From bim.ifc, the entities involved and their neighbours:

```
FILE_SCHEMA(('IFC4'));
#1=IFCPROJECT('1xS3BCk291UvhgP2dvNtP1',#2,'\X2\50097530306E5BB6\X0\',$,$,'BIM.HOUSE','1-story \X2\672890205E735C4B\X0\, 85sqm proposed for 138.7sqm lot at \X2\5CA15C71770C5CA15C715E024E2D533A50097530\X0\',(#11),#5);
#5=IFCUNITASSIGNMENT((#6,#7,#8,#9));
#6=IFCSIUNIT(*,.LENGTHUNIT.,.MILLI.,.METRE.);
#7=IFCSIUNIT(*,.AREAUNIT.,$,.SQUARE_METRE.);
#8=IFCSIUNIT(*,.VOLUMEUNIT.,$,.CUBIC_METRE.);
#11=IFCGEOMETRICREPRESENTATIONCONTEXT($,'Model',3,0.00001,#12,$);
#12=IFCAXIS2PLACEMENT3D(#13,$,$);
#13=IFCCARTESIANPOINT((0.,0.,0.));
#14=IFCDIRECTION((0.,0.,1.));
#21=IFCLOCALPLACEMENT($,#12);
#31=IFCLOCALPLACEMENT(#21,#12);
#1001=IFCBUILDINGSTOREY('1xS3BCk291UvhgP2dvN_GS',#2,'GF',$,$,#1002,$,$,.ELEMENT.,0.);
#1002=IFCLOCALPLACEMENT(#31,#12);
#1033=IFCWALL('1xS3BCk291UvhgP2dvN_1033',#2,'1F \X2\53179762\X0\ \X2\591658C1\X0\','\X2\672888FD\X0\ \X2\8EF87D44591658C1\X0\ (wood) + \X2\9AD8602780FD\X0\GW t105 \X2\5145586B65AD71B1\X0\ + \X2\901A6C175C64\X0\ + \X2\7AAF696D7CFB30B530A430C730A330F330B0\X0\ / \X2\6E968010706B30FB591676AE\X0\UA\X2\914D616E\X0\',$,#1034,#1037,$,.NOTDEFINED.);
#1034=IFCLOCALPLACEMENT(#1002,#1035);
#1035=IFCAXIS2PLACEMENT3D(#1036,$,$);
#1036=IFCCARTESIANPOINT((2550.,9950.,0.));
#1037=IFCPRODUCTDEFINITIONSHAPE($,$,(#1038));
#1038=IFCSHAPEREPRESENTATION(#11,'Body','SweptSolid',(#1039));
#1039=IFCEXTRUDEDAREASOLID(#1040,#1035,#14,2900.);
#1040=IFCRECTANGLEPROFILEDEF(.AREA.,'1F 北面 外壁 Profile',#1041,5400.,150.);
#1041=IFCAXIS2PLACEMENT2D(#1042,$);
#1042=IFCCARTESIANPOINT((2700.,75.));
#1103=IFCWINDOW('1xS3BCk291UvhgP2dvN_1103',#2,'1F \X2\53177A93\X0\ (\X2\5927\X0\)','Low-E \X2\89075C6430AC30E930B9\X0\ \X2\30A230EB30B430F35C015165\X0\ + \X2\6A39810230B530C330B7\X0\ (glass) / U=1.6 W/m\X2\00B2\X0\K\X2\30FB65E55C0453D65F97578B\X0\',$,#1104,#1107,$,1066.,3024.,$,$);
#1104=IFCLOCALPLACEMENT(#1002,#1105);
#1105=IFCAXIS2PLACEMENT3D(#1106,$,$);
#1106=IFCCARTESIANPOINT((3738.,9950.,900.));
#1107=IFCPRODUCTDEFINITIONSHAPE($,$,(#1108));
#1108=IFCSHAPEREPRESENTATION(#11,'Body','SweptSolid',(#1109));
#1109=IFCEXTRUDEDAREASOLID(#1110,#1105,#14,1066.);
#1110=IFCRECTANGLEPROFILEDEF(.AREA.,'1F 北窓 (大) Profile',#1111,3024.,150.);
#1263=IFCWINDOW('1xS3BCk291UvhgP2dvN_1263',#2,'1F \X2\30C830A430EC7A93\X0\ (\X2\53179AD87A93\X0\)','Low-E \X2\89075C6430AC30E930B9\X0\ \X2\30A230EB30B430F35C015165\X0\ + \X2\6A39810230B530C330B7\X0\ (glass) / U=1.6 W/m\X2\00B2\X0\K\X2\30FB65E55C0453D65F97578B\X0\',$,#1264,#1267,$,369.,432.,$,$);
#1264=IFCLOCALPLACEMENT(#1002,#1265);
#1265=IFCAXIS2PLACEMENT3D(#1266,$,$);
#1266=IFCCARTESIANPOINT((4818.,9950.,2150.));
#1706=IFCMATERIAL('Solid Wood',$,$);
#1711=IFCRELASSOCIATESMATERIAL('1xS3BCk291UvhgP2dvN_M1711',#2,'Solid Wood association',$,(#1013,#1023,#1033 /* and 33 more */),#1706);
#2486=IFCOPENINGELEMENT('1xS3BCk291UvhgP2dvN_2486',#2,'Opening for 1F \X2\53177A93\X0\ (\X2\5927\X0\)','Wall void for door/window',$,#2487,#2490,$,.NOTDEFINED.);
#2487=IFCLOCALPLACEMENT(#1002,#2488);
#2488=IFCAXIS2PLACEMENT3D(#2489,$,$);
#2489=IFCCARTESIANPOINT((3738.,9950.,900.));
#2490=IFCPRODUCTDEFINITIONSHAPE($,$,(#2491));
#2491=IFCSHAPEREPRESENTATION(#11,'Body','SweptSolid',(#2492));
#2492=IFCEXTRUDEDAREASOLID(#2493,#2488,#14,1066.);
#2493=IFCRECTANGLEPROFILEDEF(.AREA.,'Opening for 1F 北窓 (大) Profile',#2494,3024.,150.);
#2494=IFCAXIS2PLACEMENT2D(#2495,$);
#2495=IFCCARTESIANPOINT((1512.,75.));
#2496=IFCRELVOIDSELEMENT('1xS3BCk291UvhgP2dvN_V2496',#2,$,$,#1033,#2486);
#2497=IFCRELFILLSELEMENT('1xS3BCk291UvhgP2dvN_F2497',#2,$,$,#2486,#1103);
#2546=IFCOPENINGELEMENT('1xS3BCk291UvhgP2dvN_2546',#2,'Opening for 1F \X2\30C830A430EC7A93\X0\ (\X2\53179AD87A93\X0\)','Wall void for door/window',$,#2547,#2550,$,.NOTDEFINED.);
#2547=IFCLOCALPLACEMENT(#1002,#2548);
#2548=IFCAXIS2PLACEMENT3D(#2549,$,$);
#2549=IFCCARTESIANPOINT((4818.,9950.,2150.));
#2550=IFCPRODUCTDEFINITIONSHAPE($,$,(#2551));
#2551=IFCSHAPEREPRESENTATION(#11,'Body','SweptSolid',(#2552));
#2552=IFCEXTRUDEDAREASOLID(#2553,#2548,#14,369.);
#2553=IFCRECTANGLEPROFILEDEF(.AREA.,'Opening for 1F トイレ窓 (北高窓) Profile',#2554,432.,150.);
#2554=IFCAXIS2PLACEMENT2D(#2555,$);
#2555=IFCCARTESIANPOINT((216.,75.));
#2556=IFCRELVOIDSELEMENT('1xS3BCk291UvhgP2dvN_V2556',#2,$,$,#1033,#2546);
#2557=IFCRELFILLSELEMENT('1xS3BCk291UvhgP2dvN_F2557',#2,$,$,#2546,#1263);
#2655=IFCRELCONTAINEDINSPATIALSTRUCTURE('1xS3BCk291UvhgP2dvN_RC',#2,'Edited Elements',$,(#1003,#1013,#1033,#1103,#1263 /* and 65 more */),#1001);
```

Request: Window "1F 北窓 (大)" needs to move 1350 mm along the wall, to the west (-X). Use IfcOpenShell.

```python
import ifcopenshell
import ifcopenshell.api.geometry
import ifcopenshell.util.placement
import ifcopenshell.util.unit

model = ifcopenshell.open("bim.ifc")
unit_scale = ifcopenshell.util.unit.calculate_unit_scale(model)

window = model.by_guid("1xS3BCk291UvhgP2dvN_1103")
opening = window.FillsVoids[0].RelatingOpeningElement
wall = opening.VoidsElements[0].RelatingBuildingElement

wall_matrix = ifcopenshell.util.placement.get_local_placement(wall.ObjectPlacement)
shift = wall_matrix[:3, 0] * -1.35 / unit_scale
before = ifcopenshell.util.placement.get_local_placement(window.ObjectPlacement)[:3, 3].copy()

# The window is not placed relative to its opening, so move both.
for product in (opening, window):
    matrix = ifcopenshell.util.placement.get_local_placement(product.ObjectPlacement)
    matrix[:3, 3] += shift
    ifcopenshell.api.geometry.edit_object_placement(model, product=product, matrix=matrix, is_si=False)

after = ifcopenshell.util.placement.get_local_placement(window.ObjectPlacement)[:3, 3]
print("window moved by", (after - before).round(3) + 0.0)

model.write("bim-out.ifc")
```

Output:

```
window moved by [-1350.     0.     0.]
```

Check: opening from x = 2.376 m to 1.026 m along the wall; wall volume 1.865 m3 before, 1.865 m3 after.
